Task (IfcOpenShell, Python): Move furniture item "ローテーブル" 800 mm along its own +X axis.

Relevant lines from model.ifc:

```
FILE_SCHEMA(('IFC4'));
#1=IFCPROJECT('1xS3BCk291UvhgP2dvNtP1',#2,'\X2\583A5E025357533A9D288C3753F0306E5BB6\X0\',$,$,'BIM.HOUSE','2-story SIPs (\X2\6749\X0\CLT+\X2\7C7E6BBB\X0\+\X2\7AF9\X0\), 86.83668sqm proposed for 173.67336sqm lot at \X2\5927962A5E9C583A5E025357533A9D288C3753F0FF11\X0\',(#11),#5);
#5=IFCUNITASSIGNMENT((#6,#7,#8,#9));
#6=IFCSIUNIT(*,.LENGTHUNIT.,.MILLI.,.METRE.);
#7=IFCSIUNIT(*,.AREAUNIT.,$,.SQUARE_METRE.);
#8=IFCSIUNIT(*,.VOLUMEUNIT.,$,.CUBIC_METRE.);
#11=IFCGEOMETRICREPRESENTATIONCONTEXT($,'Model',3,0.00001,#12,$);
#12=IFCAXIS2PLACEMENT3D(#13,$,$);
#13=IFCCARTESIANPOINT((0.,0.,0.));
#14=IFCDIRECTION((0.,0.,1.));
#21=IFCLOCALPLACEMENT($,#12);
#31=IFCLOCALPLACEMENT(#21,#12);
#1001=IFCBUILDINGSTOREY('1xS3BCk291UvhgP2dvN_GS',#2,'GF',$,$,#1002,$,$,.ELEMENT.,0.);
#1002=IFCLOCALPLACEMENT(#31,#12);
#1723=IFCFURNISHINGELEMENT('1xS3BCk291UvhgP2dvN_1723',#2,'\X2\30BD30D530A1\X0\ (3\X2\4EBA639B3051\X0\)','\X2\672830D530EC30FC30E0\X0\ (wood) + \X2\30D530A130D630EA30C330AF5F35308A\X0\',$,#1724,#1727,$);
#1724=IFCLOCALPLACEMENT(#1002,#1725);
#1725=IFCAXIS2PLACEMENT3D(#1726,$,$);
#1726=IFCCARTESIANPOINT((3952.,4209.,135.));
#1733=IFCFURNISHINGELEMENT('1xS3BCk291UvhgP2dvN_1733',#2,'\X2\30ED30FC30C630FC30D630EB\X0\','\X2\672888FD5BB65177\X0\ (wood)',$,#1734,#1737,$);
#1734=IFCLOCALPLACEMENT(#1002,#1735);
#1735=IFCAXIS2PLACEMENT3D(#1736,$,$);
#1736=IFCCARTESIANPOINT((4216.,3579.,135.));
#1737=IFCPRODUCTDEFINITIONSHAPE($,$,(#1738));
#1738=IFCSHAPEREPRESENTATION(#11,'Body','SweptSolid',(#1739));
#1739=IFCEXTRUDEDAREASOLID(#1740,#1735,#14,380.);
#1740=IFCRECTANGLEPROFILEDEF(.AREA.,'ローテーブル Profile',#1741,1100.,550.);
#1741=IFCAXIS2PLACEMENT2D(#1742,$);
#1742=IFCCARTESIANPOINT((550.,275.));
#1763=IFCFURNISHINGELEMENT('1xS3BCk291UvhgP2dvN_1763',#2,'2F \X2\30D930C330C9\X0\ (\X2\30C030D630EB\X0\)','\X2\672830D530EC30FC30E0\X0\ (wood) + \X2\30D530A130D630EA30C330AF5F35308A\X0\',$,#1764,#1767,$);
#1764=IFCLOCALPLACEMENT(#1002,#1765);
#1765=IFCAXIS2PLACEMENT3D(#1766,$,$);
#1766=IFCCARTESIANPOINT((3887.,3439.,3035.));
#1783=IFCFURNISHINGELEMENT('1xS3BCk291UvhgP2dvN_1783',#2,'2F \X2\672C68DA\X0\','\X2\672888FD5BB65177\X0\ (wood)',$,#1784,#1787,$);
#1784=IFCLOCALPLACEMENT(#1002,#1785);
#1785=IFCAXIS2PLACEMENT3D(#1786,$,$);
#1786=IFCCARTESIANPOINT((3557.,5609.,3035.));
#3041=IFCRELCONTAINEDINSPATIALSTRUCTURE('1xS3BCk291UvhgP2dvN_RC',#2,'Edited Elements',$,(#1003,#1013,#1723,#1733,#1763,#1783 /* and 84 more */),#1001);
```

```python
import ifcopenshell
import ifcopenshell.api.geometry
import ifcopenshell.util.placement

model = ifcopenshell.open("model.ifc")

item = model.by_guid("1xS3BCk291UvhgP2dvN_1733")
matrix = ifcopenshell.util.placement.get_local_placement(item.ObjectPlacement)
matrix[:3, 3] += matrix[:3, 0] * 800.0
ifcopenshell.api.geometry.edit_object_placement(model, product=item, matrix=matrix, is_si=False)

print(ifcopenshell.util.placement.get_local_placement(item.ObjectPlacement).round(3) + 0.0)

model.write("model_edited.ifc")
```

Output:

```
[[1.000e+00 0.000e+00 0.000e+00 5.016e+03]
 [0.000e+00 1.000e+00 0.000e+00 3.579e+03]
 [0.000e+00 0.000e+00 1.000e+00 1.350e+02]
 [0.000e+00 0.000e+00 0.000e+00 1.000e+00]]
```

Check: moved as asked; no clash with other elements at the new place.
